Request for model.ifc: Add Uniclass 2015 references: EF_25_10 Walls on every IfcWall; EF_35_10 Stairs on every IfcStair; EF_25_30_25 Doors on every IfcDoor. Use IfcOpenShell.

First a look at what the model holds.

```python
import ifcopenshell

model = ifcopenshell.open("model.ifc")
print(model.schema)
print("classifications:", [c.Name for c in model.by_type("IfcClassification")])
for ifc_class in ("IfcDoor", "IfcRoof", "IfcStair", "IfcWall", "IfcWindow"):
    print(ifc_class, len(model.by_type(ifc_class)))
```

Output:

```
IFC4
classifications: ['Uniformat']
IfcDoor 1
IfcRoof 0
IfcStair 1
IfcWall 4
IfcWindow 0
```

```python
import ifcopenshell
import ifcopenshell.api.classification

model = ifcopenshell.open("model.ifc")

system = ifcopenshell.api.classification.add_classification(model, classification="Uniclass 2015")

codes = {
    "IfcWall": ("EF_25_10", "Walls"),
    "IfcStair": ("EF_35_10", "Stairs"),
    "IfcDoor": ("EF_25_30_25", "Doors"),
}
for ifc_class, (code, name) in codes.items():
    products = model.by_type(ifc_class)
    ifcopenshell.api.classification.add_reference(
        model, products=products, classification=system, identification=code, name=name
    )
    print(code, len(products))

model.write("model_v2.ifc")
```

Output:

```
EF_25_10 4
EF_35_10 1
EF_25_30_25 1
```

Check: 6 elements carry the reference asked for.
